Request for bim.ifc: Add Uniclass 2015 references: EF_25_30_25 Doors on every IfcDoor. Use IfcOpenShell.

First a look at what the model holds.

```python
import ifcopenshell

model = ifcopenshell.open("bim.ifc")
print(model.schema)
print("classifications:", [c.Name for c in model.by_type("IfcClassification")])
for ifc_class in ("IfcDoor", "IfcRoof", "IfcStair", "IfcWall", "IfcWindow"):
    print(ifc_class, len(model.by_type(ifc_class)))
```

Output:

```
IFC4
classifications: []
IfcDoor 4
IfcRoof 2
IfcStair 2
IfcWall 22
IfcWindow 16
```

```python
import ifcopenshell
import ifcopenshell.api.classification

model = ifcopenshell.open("bim.ifc")

system = ifcopenshell.api.classification.add_classification(model, classification="Uniclass 2015")

codes = {
    "IfcDoor": ("EF_25_30_25", "Doors"),
}
for ifc_class, (code, name) in codes.items():
    products = model.by_type(ifc_class)
    ifcopenshell.api.classification.add_reference(
        model, products=products, classification=system, identification=code, name=name
    )
    print(code, len(products))

model.write("bim_edited.ifc")
```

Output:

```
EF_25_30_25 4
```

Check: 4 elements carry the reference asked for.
